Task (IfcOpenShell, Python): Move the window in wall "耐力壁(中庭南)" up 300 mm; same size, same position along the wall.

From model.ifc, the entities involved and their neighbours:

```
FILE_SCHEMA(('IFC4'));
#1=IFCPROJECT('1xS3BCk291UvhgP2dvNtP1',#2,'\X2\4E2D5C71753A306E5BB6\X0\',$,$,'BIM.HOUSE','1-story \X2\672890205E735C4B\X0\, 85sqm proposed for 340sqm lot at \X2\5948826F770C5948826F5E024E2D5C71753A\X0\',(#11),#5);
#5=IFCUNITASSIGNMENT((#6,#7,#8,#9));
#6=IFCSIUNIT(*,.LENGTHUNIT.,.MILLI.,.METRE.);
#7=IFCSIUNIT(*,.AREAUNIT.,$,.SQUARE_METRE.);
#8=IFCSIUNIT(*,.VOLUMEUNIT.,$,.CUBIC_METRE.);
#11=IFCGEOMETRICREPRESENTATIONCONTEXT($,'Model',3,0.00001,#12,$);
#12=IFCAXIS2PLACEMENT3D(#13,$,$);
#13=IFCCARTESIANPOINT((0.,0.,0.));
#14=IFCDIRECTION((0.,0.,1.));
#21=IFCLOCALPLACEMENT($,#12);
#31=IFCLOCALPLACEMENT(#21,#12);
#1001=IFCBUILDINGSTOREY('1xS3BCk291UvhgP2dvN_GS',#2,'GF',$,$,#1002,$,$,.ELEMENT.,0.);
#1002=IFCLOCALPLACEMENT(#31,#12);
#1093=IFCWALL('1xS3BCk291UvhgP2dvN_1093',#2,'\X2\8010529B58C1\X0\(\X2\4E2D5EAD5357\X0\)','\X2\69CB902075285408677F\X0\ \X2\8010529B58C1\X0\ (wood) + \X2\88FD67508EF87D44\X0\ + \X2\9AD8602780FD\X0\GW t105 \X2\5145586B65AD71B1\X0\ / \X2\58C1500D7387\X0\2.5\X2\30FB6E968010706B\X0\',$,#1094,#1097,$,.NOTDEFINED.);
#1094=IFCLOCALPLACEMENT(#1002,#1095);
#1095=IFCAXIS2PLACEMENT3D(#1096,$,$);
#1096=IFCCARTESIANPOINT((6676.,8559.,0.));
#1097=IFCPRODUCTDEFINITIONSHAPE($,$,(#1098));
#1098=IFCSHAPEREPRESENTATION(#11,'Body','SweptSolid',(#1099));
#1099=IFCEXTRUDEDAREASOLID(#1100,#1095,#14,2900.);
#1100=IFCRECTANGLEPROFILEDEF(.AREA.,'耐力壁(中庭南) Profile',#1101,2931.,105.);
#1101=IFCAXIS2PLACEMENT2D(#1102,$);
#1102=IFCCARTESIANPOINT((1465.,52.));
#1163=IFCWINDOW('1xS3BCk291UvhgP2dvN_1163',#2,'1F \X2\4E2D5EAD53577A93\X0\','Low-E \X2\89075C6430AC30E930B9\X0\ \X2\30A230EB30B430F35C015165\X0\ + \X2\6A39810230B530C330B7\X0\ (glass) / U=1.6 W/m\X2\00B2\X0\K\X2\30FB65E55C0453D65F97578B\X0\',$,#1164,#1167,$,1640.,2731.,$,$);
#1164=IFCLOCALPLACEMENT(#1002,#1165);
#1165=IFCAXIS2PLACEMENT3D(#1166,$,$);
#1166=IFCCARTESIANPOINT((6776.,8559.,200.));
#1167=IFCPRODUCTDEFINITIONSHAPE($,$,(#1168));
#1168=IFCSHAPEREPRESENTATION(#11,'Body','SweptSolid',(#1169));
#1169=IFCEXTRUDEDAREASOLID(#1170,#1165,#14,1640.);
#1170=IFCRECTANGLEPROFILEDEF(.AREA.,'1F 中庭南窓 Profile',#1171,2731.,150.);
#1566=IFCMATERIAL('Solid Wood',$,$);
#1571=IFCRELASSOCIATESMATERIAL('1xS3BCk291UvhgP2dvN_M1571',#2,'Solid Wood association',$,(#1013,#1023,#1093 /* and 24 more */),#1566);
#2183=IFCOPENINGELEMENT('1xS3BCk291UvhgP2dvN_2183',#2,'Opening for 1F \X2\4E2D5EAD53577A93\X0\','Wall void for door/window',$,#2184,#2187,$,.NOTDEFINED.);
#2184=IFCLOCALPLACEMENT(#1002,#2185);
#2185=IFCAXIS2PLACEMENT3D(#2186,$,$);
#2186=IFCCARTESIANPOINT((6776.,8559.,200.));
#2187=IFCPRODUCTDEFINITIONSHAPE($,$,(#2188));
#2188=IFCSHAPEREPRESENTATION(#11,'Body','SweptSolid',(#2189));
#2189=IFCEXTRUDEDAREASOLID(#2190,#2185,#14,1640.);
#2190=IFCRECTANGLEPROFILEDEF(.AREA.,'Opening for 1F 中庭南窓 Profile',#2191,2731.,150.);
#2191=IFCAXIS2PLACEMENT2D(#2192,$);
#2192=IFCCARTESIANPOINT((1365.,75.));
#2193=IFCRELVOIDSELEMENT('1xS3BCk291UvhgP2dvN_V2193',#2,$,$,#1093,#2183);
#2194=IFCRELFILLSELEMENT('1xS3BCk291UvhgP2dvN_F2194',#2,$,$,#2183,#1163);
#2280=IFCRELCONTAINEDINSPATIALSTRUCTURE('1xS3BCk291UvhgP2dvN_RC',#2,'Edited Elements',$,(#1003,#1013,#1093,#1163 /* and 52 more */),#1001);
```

```python
import numpy as np
import ifcopenshell
import ifcopenshell.api.geometry
import ifcopenshell.util.placement
import ifcopenshell.util.unit

model = ifcopenshell.open("model.ifc")
unit_scale = ifcopenshell.util.unit.calculate_unit_scale(model)

window = model.by_guid("1xS3BCk291UvhgP2dvN_1163")
opening = window.FillsVoids[0].RelatingOpeningElement
dz = 0.3 / unit_scale

shift = np.array([0.0, 0.0, dz])
# The window is not placed relative to its opening, so move both.
for product in (opening, window):
    matrix = ifcopenshell.util.placement.get_local_placement(product.ObjectPlacement)
    matrix[:3, 3] += shift
    ifcopenshell.api.geometry.edit_object_placement(model, product=product, matrix=matrix, is_si=False)

print(f"moved by {dz * unit_scale:+.3f} m")

model.write("model_rev.ifc")
```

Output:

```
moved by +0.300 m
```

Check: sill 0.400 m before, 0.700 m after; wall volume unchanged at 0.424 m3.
